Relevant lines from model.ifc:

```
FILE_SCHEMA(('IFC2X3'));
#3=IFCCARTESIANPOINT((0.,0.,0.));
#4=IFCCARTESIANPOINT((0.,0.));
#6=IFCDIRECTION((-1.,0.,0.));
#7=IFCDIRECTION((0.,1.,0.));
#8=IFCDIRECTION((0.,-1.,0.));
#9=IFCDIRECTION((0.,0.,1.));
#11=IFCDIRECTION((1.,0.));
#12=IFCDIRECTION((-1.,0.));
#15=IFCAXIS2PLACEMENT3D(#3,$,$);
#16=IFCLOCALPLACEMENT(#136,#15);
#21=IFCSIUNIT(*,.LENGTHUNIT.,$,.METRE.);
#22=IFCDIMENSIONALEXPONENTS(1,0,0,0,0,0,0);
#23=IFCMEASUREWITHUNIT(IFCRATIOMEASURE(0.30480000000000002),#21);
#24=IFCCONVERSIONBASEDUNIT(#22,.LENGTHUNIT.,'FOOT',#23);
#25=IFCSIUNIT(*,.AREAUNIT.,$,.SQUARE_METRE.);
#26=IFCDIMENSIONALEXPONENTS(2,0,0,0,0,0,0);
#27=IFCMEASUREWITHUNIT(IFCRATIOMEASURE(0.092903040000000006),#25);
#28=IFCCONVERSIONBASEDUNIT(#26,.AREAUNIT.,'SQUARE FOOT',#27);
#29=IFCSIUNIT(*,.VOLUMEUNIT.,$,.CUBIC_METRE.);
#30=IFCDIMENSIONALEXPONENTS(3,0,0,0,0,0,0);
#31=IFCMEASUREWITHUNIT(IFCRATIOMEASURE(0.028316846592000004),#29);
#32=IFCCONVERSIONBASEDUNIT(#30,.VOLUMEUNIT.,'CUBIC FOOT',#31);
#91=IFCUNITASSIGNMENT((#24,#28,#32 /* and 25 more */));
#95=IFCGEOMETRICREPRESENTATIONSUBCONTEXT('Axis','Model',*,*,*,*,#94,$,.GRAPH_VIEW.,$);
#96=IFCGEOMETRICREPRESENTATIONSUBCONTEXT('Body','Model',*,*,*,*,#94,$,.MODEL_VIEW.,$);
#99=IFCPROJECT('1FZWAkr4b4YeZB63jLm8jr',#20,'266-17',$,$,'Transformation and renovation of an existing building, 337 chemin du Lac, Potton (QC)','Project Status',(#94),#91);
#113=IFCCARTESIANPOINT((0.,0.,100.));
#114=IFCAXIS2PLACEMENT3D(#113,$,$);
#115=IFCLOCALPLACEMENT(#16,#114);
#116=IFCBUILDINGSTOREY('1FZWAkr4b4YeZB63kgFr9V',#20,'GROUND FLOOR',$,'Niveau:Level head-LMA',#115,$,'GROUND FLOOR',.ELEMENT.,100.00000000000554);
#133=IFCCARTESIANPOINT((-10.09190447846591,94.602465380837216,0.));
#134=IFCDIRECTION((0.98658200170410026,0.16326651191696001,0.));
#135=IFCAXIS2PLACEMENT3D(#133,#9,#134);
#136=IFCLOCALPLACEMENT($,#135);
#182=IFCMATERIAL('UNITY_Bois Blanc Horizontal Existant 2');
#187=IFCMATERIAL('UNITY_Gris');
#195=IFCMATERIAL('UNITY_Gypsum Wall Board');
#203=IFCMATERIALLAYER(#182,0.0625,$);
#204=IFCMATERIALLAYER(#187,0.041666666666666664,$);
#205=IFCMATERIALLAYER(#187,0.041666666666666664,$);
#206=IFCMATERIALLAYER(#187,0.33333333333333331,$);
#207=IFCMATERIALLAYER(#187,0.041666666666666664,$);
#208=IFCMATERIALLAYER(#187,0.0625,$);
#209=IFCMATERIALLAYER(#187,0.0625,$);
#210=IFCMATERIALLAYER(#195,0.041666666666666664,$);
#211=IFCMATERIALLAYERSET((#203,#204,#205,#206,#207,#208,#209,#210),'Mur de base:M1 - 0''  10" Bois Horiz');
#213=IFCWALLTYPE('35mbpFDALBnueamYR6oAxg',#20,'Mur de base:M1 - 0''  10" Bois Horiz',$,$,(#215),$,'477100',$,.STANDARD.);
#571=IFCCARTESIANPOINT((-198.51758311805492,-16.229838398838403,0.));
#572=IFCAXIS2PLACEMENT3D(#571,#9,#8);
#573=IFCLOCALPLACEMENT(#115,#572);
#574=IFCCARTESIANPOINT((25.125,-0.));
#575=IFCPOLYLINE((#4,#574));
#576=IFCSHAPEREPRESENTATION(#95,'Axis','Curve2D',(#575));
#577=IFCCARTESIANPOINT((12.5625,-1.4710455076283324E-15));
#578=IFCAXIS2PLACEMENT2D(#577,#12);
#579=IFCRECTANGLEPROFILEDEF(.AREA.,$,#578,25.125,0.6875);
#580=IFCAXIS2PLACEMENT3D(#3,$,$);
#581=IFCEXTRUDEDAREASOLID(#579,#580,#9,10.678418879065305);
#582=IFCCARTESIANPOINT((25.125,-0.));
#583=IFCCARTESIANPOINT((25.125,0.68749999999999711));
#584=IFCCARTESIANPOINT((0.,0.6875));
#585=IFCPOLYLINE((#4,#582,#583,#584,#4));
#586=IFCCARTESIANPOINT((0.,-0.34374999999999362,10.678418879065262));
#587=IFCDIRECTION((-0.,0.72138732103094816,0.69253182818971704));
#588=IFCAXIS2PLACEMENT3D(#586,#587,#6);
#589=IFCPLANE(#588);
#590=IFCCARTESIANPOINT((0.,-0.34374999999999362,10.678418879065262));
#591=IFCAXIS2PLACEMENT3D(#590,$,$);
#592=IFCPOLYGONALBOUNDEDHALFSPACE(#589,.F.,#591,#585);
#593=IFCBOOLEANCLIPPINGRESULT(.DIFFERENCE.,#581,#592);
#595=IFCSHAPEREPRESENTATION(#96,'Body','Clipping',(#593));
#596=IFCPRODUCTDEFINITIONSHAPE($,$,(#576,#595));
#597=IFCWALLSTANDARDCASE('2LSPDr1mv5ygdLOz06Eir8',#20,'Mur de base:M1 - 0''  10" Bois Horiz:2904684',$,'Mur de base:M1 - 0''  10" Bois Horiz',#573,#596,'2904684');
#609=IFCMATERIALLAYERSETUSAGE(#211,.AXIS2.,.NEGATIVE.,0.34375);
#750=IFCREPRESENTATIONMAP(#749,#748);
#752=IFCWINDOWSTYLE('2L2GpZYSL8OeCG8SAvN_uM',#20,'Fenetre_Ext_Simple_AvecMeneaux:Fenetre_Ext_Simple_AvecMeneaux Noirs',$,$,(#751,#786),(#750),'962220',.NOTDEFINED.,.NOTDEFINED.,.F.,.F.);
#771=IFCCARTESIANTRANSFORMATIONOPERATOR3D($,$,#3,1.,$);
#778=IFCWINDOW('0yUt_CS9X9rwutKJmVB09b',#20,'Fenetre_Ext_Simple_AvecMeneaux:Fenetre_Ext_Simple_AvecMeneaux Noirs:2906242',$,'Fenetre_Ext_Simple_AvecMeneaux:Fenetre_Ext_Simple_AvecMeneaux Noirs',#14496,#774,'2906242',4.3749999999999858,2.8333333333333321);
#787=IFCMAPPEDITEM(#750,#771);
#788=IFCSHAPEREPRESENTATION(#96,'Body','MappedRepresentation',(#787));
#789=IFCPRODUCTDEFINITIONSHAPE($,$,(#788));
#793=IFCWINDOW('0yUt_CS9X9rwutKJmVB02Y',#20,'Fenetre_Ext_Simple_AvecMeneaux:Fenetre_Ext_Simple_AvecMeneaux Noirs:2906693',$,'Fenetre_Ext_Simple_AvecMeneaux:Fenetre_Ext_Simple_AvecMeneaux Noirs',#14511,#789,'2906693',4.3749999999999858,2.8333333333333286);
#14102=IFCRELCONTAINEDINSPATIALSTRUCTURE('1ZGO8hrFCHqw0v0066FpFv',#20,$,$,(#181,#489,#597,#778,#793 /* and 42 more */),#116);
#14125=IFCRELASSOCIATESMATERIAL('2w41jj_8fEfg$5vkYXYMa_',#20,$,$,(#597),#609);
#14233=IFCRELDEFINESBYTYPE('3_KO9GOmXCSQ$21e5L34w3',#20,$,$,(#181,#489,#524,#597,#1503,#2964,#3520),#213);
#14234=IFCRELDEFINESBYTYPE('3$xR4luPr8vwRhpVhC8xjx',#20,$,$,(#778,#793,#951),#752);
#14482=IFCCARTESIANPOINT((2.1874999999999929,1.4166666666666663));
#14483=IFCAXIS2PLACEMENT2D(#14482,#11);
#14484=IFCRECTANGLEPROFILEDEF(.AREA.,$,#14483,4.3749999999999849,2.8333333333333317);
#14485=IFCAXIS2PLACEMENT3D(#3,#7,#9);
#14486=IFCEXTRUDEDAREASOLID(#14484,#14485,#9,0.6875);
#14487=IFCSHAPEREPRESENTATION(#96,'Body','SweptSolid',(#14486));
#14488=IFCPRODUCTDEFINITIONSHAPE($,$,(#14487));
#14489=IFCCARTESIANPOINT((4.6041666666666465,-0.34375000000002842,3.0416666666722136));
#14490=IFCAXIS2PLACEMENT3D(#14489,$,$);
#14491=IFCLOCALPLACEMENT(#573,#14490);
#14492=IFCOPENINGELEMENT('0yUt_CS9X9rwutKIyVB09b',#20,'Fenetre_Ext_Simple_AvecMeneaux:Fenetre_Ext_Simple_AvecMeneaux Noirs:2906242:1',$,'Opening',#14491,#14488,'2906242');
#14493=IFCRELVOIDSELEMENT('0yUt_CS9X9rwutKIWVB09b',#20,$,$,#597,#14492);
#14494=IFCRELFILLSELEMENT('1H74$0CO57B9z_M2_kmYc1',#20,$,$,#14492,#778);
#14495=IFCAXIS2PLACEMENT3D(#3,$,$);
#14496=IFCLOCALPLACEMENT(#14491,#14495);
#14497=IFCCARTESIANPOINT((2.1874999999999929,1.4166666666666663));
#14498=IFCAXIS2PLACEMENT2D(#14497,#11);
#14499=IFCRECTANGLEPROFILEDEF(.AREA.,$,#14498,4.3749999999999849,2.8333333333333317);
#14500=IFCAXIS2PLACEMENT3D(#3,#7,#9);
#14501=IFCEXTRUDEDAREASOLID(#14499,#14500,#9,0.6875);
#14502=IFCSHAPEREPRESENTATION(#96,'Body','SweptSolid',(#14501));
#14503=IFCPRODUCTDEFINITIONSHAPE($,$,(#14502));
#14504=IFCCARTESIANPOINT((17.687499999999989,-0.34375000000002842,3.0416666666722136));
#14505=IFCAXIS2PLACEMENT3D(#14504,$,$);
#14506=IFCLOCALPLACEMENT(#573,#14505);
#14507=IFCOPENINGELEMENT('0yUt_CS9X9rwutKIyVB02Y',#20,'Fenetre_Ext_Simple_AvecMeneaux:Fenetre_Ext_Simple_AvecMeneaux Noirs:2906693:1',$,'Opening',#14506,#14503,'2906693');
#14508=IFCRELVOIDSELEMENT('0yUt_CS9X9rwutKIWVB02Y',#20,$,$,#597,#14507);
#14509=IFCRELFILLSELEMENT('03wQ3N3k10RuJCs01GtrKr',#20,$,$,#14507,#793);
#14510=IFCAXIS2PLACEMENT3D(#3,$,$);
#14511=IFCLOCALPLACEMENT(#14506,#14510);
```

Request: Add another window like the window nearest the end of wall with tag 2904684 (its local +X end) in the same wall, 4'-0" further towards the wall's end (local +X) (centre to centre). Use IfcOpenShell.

```python
import ifcopenshell
import ifcopenshell.api.feature
import ifcopenshell.api.geometry
import ifcopenshell.api.root
import ifcopenshell.geom
import ifcopenshell.util.element
import ifcopenshell.util.placement
import ifcopenshell.util.shape
import ifcopenshell.util.unit

model = ifcopenshell.open("model.ifc")
unit_scale = ifcopenshell.util.unit.calculate_unit_scale(model)
settings = ifcopenshell.geom.settings()


def volume(element):
    """Net volume in cubic metres, openings subtracted."""
    shape = ifcopenshell.geom.create_shape(settings, element)
    return ifcopenshell.util.shape.get_volume(shape.geometry)


def reuse_history(source, copy):
    """copy_class also copies each property set's owner history, people and application; keep the originals."""
    for rel in copy.IsDefinedBy:
        if rel.is_a("IfcRelDefinesByProperties") and (history := rel.RelatingPropertyDefinition.OwnerHistory):
            rel.RelatingPropertyDefinition.OwnerHistory = source.OwnerHistory
            ifcopenshell.util.element.remove_deep2(model, history)


window = model.by_id(793)
opening = window.FillsVoids[0].RelatingOpeningElement
wall = opening.VoidsElements[0].RelatingBuildingElement
before = volume(wall)
shift = ifcopenshell.util.placement.get_local_placement(wall.ObjectPlacement)[:3, 0] * 48 * 0.0254 / unit_scale

# copy_class copies the void relationship, type, container and properties, but no geometry.
new_opening = ifcopenshell.api.root.copy_class(model, product=opening)
new_opening.Representation = ifcopenshell.util.element.copy_deep(
    model, opening.Representation, exclude=["IfcGeometricRepresentationContext", "IfcRepresentationMap"]
)
new_opening.Name = "Fenetre_Ext_Simple_AvecMeneaux:Fenetre_Ext_Simple_AvecMeneaux Noirs"
new_opening.Tag = None
new_window = ifcopenshell.api.root.copy_class(model, product=window)
new_window.Representation = ifcopenshell.util.element.copy_deep(
    model, window.Representation, exclude=["IfcGeometricRepresentationContext", "IfcRepresentationMap"]
)
new_window.Name = "Fenetre_Ext_Simple_AvecMeneaux:Fenetre_Ext_Simple_AvecMeneaux Noirs"
new_window.Tag = None
reuse_history(window, new_window)
fills = ifcopenshell.api.feature.add_filling(model, opening=new_opening, element=new_window)
fills.OwnerHistory = new_window.OwnerHistory  # required in IFC2X3

for old, new in ((opening, new_opening), (window, new_window)):
    matrix = ifcopenshell.util.placement.get_local_placement(old.ObjectPlacement)
    matrix[:3, 3] += shift
    ifcopenshell.api.geometry.edit_object_placement(model, product=new, matrix=matrix, is_si=False)

after = volume(wall)

print(f"wall volume {before:.3f} -> {after:.3f} m3")

model.write("model_v2.ifc")
```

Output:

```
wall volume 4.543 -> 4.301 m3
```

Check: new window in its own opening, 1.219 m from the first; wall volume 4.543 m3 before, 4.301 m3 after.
